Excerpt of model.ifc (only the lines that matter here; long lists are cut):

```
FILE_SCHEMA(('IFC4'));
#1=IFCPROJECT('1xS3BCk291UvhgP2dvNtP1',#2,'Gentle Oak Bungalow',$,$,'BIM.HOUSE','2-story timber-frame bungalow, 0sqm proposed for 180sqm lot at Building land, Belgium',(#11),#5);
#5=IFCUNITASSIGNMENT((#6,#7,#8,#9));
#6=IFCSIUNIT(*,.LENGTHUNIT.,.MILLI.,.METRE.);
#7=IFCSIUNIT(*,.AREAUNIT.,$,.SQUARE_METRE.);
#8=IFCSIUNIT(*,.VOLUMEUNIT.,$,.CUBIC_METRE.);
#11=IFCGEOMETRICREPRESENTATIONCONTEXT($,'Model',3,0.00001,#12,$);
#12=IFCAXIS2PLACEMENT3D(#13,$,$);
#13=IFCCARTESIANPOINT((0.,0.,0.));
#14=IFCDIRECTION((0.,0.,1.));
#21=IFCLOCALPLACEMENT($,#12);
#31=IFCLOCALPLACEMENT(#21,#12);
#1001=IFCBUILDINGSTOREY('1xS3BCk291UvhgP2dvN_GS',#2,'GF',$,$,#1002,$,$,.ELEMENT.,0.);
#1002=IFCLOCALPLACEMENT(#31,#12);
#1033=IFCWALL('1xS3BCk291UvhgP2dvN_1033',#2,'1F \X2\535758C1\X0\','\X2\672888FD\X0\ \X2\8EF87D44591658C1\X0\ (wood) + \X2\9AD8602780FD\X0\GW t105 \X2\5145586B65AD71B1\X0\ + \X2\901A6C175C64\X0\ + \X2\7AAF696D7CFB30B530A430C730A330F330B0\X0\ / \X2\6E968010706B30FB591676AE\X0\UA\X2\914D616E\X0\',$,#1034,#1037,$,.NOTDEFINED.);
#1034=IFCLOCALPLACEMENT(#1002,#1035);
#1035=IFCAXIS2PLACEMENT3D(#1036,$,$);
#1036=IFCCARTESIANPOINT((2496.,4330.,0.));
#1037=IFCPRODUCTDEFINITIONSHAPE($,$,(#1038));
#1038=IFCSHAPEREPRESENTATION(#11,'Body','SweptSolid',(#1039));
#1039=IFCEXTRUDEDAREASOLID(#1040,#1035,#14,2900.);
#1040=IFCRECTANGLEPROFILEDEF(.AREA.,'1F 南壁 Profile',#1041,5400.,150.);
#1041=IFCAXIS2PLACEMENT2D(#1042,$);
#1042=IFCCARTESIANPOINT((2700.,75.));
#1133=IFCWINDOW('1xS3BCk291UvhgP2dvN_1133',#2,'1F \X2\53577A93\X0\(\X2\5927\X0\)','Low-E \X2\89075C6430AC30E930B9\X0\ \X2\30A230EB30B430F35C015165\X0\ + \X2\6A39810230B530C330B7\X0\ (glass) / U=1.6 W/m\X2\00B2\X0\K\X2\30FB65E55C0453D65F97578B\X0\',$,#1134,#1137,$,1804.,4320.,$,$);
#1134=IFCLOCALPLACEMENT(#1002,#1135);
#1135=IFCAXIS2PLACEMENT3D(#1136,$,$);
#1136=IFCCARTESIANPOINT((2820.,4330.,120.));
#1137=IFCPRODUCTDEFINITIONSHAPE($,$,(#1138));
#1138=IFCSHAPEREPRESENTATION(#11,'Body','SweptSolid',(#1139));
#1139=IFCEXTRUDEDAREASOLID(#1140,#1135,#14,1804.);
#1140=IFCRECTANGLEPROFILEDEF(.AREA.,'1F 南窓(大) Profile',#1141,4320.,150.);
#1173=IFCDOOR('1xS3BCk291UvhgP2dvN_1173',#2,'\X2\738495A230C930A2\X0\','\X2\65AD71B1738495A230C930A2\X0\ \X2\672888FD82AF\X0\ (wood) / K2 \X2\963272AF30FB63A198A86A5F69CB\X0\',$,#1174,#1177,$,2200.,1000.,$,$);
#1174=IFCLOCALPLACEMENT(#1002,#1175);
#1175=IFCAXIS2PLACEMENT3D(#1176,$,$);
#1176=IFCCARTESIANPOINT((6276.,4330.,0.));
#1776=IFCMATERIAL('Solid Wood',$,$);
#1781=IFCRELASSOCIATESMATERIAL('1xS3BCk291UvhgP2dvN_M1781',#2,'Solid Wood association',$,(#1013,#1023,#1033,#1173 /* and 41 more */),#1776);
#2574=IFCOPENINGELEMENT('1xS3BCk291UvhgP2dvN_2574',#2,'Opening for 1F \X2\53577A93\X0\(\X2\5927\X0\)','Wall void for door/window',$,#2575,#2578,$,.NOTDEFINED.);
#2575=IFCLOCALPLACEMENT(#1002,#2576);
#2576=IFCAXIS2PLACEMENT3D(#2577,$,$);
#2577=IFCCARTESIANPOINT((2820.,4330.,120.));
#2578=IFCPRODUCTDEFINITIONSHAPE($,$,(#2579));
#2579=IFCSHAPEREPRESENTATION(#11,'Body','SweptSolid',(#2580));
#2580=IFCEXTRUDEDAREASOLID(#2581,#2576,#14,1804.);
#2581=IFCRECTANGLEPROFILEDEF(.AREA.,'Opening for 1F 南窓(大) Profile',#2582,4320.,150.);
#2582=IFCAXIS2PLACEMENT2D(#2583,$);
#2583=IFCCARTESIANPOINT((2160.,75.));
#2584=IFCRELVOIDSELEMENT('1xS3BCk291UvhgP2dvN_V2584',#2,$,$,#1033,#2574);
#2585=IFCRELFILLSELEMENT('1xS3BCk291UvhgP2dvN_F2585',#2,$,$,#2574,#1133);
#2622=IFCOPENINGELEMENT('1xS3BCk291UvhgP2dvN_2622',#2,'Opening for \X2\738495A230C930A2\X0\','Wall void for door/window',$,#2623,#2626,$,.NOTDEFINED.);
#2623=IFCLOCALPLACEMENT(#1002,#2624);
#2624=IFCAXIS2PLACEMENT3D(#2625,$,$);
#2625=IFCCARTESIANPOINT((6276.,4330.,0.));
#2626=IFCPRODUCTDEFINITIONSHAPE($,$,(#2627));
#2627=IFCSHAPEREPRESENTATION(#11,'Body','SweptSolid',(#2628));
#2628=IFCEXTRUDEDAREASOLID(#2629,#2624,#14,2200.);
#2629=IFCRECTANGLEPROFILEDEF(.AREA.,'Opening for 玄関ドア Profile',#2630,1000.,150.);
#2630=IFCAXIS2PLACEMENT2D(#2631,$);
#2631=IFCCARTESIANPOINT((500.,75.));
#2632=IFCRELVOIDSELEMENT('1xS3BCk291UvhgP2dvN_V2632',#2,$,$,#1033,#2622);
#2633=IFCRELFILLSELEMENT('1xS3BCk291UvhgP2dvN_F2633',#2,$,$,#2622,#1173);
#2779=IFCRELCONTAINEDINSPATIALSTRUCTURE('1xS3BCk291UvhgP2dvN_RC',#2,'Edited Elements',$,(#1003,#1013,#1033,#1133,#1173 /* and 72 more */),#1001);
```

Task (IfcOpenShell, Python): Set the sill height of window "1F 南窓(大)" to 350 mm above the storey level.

```python
import numpy as np
import ifcopenshell
import ifcopenshell.api.geometry
import ifcopenshell.geom
import ifcopenshell.util.element
import ifcopenshell.util.placement
import ifcopenshell.util.shape
import ifcopenshell.util.unit

model = ifcopenshell.open("model.ifc")
unit_scale = ifcopenshell.util.unit.calculate_unit_scale(model)

window = model.by_guid("1xS3BCk291UvhgP2dvN_1133")
opening = window.FillsVoids[0].RelatingOpeningElement
storey = ifcopenshell.util.element.get_container(window, ifc_class="IfcBuildingStorey")
level = ifcopenshell.util.placement.get_local_placement(storey.ObjectPlacement)[2, 3]

# The opening's origin need not be at the sill, so measure its lowest point.
shape = ifcopenshell.geom.create_shape(ifcopenshell.geom.settings(), opening)
bottom = ifcopenshell.util.shape.get_shape_bottom_elevation(shape, shape.geometry) / unit_scale
dz = level + 0.35 / unit_scale - bottom

shift = np.array([0.0, 0.0, dz])
# The window is not placed relative to its opening, so move both.
for product in (opening, window):
    matrix = ifcopenshell.util.placement.get_local_placement(product.ObjectPlacement)
    matrix[:3, 3] += shift
    ifcopenshell.api.geometry.edit_object_placement(model, product=product, matrix=matrix, is_si=False)

print(f"moved by {dz * unit_scale:+.3f} m")

model.write("model_edited.ifc")
```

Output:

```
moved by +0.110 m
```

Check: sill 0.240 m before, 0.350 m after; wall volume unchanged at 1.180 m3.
